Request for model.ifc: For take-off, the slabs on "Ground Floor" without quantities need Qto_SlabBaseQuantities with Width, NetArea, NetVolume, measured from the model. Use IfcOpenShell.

First a look at what the model holds.

```python
import ifcopenshell
import ifcopenshell.util.element
import ifcopenshell.util.unit

model = ifcopenshell.open("model.ifc")
print(model.schema)
for unit_type in ("LENGTHUNIT", "AREAUNIT", "VOLUMEUNIT"):
    print(unit_type, ifcopenshell.util.unit.calculate_unit_scale(model, unit_type))
storey = next(s for s in model.by_type("IfcBuildingStorey") if s.Name == "Ground Floor")
slabs = [e for e in ifcopenshell.util.element.get_decomposition(storey) if e.is_a("IfcSlab")]
for e in sorted(slabs, key=lambda e: e.id()):
    print(e.id(), e.is_a(), e.Name, list(ifcopenshell.util.element.get_psets(e, qtos_only=True)), sep=" | ")
```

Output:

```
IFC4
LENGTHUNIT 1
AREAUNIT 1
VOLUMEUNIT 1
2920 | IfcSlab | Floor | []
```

```python
import ifcopenshell
import ifcopenshell.api.pset
import ifcopenshell.geom
import ifcopenshell.util.element
import ifcopenshell.util.shape
import ifcopenshell.util.unit

model = ifcopenshell.open("model.ifc")
unit_scale = ifcopenshell.util.unit.calculate_unit_scale(model)
area_scale = ifcopenshell.util.unit.calculate_unit_scale(model, "AREAUNIT")
volume_scale = ifcopenshell.util.unit.calculate_unit_scale(model, "VOLUMEUNIT")
settings = ifcopenshell.geom.settings()

storey = next(s for s in model.by_type("IfcBuildingStorey") if s.Name == "Ground Floor")
slabs = [e for e in ifcopenshell.util.element.get_decomposition(storey) if e.is_a("IfcSlab")]

for e in sorted(slabs, key=lambda e: e.id()):
    if ifcopenshell.util.element.get_psets(e, qtos_only=True, should_inherit=False):
        continue
    # Geometry comes back in metres, in the element's own axes.
    shape = ifcopenshell.geom.create_shape(settings, e)
    values = {
        "Width": ifcopenshell.util.shape.get_z(shape.geometry) / unit_scale,
        "NetArea": ifcopenshell.util.shape.get_footprint_area(shape.geometry) / area_scale,
        "NetVolume": ifcopenshell.util.shape.get_volume(shape.geometry) / volume_scale,
    }
    qto = ifcopenshell.api.pset.add_qto(model, product=e, name="Qto_SlabBaseQuantities")
    ifcopenshell.api.pset.edit_qto(model, qto=qto, properties=values)
    print(e.id(), {k: round(v, 3) for k, v in values.items()})

model.write("model_rev.ifc")
```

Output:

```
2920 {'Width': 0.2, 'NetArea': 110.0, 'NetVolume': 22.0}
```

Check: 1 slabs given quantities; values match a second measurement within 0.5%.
